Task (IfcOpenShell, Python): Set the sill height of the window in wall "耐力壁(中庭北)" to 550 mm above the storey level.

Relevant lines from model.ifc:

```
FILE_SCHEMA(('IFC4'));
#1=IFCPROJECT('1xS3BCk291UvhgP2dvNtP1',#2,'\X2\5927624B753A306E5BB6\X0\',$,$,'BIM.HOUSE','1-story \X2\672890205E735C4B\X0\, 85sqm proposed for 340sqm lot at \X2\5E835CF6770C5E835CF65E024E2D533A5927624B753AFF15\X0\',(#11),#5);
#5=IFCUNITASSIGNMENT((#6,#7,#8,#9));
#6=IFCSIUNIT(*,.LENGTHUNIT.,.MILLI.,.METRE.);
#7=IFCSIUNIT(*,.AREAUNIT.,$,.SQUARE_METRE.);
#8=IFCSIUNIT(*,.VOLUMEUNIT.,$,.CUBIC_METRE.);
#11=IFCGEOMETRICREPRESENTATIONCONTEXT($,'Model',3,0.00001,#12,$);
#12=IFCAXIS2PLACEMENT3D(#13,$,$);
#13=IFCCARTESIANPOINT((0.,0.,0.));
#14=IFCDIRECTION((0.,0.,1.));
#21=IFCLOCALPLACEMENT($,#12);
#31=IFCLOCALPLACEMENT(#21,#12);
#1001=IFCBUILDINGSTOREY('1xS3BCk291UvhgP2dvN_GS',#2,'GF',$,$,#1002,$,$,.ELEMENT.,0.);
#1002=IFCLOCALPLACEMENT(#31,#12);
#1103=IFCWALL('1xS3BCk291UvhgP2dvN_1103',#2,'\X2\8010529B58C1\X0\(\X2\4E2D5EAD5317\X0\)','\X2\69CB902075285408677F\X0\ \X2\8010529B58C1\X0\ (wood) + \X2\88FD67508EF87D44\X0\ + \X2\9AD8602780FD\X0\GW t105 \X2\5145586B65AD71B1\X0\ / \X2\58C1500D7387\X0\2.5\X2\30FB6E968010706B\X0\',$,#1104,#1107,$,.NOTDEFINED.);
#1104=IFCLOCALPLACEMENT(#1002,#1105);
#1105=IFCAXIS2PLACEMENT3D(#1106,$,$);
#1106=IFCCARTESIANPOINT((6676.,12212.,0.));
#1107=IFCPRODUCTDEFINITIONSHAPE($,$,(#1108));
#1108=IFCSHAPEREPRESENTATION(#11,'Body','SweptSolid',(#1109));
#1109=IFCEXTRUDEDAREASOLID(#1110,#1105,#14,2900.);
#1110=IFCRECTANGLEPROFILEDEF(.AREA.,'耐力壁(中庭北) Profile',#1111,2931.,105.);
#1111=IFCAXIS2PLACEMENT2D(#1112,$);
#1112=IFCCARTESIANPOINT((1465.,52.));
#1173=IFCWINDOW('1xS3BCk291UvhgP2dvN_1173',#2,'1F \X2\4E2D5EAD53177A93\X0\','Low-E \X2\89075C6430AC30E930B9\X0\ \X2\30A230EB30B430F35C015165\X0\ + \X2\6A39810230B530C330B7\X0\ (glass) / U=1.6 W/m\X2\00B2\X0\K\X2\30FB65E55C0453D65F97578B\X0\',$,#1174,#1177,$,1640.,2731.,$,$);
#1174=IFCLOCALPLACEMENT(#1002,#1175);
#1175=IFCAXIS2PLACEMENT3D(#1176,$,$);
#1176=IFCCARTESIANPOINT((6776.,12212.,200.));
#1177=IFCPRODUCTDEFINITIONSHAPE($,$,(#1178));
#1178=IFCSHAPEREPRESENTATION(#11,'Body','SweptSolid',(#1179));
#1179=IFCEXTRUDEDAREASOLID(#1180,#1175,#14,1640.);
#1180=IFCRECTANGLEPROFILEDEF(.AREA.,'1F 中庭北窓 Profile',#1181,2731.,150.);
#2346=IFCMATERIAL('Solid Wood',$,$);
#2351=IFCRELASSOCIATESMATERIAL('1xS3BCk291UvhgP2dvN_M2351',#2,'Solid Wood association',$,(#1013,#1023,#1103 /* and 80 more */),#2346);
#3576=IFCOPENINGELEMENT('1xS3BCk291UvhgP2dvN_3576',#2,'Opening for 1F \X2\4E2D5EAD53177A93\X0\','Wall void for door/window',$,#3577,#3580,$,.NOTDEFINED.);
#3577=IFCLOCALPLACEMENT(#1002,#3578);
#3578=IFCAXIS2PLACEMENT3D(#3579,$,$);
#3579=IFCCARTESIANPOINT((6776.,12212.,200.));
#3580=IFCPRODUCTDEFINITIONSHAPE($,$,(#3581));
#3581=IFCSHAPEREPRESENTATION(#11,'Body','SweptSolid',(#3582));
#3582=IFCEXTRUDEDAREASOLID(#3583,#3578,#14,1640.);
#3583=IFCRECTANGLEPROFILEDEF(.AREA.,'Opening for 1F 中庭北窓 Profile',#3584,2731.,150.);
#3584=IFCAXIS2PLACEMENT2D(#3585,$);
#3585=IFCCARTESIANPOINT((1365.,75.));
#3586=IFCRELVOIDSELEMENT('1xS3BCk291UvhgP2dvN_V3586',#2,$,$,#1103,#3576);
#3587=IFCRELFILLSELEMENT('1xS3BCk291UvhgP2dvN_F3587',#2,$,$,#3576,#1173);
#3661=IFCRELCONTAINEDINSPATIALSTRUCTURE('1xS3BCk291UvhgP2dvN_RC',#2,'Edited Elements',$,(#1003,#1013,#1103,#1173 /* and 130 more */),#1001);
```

```python
import numpy as np
import ifcopenshell
import ifcopenshell.api.geometry
import ifcopenshell.geom
import ifcopenshell.util.element
import ifcopenshell.util.placement
import ifcopenshell.util.shape
import ifcopenshell.util.unit

model = ifcopenshell.open("model.ifc")
unit_scale = ifcopenshell.util.unit.calculate_unit_scale(model)

window = model.by_id(1173)
opening = window.FillsVoids[0].RelatingOpeningElement
storey = ifcopenshell.util.element.get_container(window, ifc_class="IfcBuildingStorey")
level = ifcopenshell.util.placement.get_local_placement(storey.ObjectPlacement)[2, 3]

# The opening's origin need not be at the sill, so measure its lowest point.
shape = ifcopenshell.geom.create_shape(ifcopenshell.geom.settings(), opening)
bottom = ifcopenshell.util.shape.get_shape_bottom_elevation(shape, shape.geometry) / unit_scale
dz = level + 550.0 - bottom

shift = np.array([0.0, 0.0, dz])
# The window is not placed relative to its opening, so move both.
for product in (opening, window):
    matrix = ifcopenshell.util.placement.get_local_placement(product.ObjectPlacement)
    matrix[:3, 3] += shift
    ifcopenshell.api.geometry.edit_object_placement(model, product=product, matrix=matrix, is_si=False)

print(f"moved by {dz * unit_scale:+.3f} m")

model.write("model_v2.ifc")
```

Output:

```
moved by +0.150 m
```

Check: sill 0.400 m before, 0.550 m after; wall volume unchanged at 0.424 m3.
